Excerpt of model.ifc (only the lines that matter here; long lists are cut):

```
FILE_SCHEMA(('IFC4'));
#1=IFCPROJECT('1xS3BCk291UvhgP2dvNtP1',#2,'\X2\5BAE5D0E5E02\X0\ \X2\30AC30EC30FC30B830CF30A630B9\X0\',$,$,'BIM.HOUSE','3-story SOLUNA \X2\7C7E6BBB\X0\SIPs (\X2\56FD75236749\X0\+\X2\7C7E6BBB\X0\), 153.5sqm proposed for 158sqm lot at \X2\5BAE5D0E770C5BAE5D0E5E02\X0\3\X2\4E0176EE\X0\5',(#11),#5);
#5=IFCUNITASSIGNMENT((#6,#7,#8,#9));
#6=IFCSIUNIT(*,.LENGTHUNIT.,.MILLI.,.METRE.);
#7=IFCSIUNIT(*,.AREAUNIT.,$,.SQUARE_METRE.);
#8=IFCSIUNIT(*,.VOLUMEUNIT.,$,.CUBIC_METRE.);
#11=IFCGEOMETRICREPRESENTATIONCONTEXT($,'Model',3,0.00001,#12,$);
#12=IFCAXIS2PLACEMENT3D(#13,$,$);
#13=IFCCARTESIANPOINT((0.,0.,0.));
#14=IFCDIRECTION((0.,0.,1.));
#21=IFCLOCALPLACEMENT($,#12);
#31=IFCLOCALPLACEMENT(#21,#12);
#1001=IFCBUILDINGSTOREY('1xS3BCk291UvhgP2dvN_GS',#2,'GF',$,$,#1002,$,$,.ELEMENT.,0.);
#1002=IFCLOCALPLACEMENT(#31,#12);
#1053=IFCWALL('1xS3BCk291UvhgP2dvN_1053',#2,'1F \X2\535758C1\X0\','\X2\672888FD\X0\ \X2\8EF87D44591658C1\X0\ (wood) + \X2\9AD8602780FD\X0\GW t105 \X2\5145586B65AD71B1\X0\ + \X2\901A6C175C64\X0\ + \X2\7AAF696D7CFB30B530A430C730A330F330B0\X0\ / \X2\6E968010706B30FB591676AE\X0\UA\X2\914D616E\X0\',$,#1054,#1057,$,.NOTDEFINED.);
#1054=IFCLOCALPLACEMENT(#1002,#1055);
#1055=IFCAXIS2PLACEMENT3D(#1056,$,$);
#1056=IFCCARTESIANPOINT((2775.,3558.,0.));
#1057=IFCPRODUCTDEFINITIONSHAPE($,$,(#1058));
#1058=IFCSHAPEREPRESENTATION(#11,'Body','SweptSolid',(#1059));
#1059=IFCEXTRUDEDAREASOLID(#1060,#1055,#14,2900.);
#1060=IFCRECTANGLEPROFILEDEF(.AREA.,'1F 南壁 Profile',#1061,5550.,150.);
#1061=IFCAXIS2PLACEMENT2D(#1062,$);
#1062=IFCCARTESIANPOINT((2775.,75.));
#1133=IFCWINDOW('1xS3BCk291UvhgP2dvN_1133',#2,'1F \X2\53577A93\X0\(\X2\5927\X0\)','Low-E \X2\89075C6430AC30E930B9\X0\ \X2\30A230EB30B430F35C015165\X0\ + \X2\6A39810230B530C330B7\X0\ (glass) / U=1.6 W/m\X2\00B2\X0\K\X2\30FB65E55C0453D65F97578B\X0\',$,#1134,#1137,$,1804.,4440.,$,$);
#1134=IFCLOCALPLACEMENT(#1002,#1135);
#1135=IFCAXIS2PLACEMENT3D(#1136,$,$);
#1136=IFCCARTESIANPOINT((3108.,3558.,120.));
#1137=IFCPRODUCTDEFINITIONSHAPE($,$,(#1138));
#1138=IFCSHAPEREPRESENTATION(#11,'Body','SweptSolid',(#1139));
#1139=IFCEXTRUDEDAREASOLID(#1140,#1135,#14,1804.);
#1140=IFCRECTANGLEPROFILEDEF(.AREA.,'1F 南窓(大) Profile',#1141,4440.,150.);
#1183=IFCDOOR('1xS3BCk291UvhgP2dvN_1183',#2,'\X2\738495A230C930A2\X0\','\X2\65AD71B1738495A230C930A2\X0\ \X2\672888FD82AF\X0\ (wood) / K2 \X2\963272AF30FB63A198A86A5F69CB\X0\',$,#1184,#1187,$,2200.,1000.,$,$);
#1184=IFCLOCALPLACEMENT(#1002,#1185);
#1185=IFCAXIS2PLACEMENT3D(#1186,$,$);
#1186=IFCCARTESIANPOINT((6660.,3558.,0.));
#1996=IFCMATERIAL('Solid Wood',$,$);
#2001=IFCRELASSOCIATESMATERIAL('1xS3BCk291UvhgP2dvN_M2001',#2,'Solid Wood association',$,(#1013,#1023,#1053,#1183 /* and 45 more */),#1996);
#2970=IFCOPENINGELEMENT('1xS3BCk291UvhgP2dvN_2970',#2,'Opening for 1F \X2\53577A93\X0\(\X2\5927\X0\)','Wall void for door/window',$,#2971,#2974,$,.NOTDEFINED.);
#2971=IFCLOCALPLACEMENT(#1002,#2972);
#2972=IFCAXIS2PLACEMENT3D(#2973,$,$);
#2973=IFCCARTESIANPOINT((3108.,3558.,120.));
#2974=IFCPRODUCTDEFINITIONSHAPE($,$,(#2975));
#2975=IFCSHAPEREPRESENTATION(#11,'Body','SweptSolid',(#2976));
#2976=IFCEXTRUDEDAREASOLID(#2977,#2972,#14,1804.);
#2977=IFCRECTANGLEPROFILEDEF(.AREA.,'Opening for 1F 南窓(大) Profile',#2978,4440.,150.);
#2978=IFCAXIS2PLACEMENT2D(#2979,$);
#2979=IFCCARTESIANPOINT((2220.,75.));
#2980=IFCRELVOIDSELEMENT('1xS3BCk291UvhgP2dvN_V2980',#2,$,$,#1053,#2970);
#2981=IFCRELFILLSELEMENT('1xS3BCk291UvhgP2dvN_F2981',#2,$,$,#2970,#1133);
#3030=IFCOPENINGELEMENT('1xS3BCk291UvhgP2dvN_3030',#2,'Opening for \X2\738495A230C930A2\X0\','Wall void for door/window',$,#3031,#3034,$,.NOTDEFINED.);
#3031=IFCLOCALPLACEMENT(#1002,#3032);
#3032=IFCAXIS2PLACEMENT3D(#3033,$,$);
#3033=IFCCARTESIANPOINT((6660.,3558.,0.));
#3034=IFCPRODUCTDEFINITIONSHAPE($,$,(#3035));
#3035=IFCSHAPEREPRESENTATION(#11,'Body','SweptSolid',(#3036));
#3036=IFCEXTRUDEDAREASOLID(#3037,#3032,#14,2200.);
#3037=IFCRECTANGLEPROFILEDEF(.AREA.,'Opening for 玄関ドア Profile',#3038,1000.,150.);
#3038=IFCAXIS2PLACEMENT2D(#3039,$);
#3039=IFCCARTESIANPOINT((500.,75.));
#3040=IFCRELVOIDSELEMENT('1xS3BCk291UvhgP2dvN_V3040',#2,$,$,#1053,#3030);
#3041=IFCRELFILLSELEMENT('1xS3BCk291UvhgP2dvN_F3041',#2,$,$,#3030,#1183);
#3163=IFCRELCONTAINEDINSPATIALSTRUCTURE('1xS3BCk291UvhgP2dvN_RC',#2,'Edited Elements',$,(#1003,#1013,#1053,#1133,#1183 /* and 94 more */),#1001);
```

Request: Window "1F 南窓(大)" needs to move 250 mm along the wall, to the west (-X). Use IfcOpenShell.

```python
import ifcopenshell
import ifcopenshell.api.geometry
import ifcopenshell.util.placement
import ifcopenshell.util.unit

model = ifcopenshell.open("model.ifc")
unit_scale = ifcopenshell.util.unit.calculate_unit_scale(model)

window = model.by_guid("1xS3BCk291UvhgP2dvN_1133")
opening = window.FillsVoids[0].RelatingOpeningElement
wall = opening.VoidsElements[0].RelatingBuildingElement

wall_matrix = ifcopenshell.util.placement.get_local_placement(wall.ObjectPlacement)
shift = wall_matrix[:3, 0] * -0.25 / unit_scale
before = ifcopenshell.util.placement.get_local_placement(window.ObjectPlacement)[:3, 3].copy()

# The window is not placed relative to its opening, so move both.
for product in (opening, window):
    matrix = ifcopenshell.util.placement.get_local_placement(product.ObjectPlacement)
    matrix[:3, 3] += shift
    ifcopenshell.api.geometry.edit_object_placement(model, product=product, matrix=matrix, is_si=False)

after = ifcopenshell.util.placement.get_local_placement(window.ObjectPlacement)[:3, 3]
print("window moved by", (after - before).round(3) + 0.0)

model.write("model_updated.ifc")
```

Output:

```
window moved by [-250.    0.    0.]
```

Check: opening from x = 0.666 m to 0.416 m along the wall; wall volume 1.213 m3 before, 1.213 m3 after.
